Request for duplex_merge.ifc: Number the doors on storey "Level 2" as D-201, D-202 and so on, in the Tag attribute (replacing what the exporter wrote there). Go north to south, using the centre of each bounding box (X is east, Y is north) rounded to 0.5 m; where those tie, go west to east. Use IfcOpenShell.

First a look at what the model holds.

```python
import ifcopenshell
import ifcopenshell.util.element
import ifcopenshell.util.placement

model = ifcopenshell.open("duplex_merge.ifc")
print(model.schema)
storey = next(s for s in model.by_type("IfcBuildingStorey") if s.Name == "Level 2")
doors = [e for e in ifcopenshell.util.element.get_decomposition(storey) if e.is_a("IfcDoor")]
for e in sorted(doors, key=lambda e: e.id()):
    origin = ifcopenshell.util.placement.get_local_placement(e.ObjectPlacement)[:3, 3]
    print(e.id(), e.Tag, e.Name, origin.round(2) + 0.0, sep=" | ")
```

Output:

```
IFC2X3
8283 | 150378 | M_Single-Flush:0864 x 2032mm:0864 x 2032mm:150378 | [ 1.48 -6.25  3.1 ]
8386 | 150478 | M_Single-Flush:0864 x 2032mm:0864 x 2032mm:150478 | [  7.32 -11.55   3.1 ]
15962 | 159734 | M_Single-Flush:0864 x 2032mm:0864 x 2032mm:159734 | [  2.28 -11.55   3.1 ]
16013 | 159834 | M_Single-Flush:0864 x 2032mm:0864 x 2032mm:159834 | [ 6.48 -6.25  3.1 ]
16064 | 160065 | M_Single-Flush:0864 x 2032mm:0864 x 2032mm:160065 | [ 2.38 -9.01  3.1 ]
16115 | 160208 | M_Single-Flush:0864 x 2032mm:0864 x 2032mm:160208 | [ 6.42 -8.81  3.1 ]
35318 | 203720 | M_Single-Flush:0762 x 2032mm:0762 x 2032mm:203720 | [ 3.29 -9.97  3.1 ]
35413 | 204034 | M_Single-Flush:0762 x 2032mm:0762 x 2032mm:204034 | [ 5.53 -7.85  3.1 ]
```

```python
import ifcopenshell
import ifcopenshell.geom
import ifcopenshell.util.element
import ifcopenshell.util.shape

model = ifcopenshell.open("duplex_merge.ifc")
settings = ifcopenshell.geom.settings()
settings.set("use-world-coords", True)


def centre(element):
    shape = ifcopenshell.geom.create_shape(settings, element)
    return ifcopenshell.util.shape.get_bbox_centroid(shape.geometry)


storey = next(s for s in model.by_type("IfcBuildingStorey") if s.Name == "Level 2")
doors = [e for e in ifcopenshell.util.element.get_decomposition(storey) if e.is_a("IfcDoor")]

# Insertion points can sit at a corner or the storey origin, so sort by the geometry (in metres).
centres = {e: centre(e) for e in doors}
doors.sort(key=lambda e: (-round(centres[e][1] / 0.5), centres[e][0]))

for i, e in enumerate(doors, start=1):
    number = f"D-2{i:02d}"
    e.Tag = number
    print(e.id(), number)

model.write("duplex_merge-out.ifc")
```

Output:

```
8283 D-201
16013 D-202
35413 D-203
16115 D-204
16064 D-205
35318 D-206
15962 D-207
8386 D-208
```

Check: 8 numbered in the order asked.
